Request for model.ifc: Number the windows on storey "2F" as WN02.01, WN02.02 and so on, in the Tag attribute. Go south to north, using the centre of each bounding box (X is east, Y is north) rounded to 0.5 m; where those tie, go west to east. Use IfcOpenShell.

First a look at what the model holds.

```python
import ifcopenshell
import ifcopenshell.util.element
import ifcopenshell.util.placement

model = ifcopenshell.open("model.ifc")
print(model.schema)
storey = next(s for s in model.by_type("IfcBuildingStorey") if s.Name == "2F")
windows = [e for e in ifcopenshell.util.element.get_decomposition(storey) if e.is_a("IfcWindow")]
for e in sorted(windows, key=lambda e: e.id()):
    origin = ifcopenshell.util.placement.get_local_placement(e.ObjectPlacement)[:3, 3]
    print(e.id(), e.Tag, e.Name, origin.round(2) + 0.0, sep=" | ")
```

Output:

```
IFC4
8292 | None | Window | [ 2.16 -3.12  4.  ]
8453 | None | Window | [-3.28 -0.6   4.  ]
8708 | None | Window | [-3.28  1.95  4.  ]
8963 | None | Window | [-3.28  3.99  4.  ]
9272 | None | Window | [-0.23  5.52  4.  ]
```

```python
import ifcopenshell
import ifcopenshell.geom
import ifcopenshell.util.element
import ifcopenshell.util.shape

model = ifcopenshell.open("model.ifc")
settings = ifcopenshell.geom.settings()
settings.set("use-world-coords", True)


def centre(element):
    shape = ifcopenshell.geom.create_shape(settings, element)
    return ifcopenshell.util.shape.get_bbox_centroid(shape.geometry)


storey = next(s for s in model.by_type("IfcBuildingStorey") if s.Name == "2F")
windows = [e for e in ifcopenshell.util.element.get_decomposition(storey) if e.is_a("IfcWindow")]

# Insertion points can sit at a corner or the storey origin, so sort by the geometry (in metres).
centres = {e: centre(e) for e in windows}
windows.sort(key=lambda e: (round(centres[e][1] / 0.5), centres[e][0]))

for i, e in enumerate(windows, start=1):
    number = f"WN02.{i:02d}"
    e.Tag = number
    print(e.id(), number)

model.write("model_edited.ifc")
```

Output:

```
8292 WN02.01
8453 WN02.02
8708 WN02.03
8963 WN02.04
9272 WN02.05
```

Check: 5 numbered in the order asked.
